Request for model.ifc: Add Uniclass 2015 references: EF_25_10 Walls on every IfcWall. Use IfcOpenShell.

First a look at what the model holds.

```python
import ifcopenshell

model = ifcopenshell.open("model.ifc")
print(model.schema)
print("classifications:", [c.Name for c in model.by_type("IfcClassification")])
for ifc_class in ("IfcDoor", "IfcRoof", "IfcStair", "IfcWall", "IfcWindow"):
    print(ifc_class, len(model.by_type(ifc_class)))
```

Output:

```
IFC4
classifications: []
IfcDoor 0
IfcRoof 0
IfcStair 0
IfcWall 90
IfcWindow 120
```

```python
import ifcopenshell
import ifcopenshell.api.classification

model = ifcopenshell.open("model.ifc")

system = ifcopenshell.api.classification.add_classification(model, classification="Uniclass 2015")

codes = {
    "IfcWall": ("EF_25_10", "Walls"),
}
for ifc_class, (code, name) in codes.items():
    products = model.by_type(ifc_class)
    ifcopenshell.api.classification.add_reference(
        model, products=products, classification=system, identification=code, name=name
    )
    print(code, len(products))

model.write("model-out.ifc")
```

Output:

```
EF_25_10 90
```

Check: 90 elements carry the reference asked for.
